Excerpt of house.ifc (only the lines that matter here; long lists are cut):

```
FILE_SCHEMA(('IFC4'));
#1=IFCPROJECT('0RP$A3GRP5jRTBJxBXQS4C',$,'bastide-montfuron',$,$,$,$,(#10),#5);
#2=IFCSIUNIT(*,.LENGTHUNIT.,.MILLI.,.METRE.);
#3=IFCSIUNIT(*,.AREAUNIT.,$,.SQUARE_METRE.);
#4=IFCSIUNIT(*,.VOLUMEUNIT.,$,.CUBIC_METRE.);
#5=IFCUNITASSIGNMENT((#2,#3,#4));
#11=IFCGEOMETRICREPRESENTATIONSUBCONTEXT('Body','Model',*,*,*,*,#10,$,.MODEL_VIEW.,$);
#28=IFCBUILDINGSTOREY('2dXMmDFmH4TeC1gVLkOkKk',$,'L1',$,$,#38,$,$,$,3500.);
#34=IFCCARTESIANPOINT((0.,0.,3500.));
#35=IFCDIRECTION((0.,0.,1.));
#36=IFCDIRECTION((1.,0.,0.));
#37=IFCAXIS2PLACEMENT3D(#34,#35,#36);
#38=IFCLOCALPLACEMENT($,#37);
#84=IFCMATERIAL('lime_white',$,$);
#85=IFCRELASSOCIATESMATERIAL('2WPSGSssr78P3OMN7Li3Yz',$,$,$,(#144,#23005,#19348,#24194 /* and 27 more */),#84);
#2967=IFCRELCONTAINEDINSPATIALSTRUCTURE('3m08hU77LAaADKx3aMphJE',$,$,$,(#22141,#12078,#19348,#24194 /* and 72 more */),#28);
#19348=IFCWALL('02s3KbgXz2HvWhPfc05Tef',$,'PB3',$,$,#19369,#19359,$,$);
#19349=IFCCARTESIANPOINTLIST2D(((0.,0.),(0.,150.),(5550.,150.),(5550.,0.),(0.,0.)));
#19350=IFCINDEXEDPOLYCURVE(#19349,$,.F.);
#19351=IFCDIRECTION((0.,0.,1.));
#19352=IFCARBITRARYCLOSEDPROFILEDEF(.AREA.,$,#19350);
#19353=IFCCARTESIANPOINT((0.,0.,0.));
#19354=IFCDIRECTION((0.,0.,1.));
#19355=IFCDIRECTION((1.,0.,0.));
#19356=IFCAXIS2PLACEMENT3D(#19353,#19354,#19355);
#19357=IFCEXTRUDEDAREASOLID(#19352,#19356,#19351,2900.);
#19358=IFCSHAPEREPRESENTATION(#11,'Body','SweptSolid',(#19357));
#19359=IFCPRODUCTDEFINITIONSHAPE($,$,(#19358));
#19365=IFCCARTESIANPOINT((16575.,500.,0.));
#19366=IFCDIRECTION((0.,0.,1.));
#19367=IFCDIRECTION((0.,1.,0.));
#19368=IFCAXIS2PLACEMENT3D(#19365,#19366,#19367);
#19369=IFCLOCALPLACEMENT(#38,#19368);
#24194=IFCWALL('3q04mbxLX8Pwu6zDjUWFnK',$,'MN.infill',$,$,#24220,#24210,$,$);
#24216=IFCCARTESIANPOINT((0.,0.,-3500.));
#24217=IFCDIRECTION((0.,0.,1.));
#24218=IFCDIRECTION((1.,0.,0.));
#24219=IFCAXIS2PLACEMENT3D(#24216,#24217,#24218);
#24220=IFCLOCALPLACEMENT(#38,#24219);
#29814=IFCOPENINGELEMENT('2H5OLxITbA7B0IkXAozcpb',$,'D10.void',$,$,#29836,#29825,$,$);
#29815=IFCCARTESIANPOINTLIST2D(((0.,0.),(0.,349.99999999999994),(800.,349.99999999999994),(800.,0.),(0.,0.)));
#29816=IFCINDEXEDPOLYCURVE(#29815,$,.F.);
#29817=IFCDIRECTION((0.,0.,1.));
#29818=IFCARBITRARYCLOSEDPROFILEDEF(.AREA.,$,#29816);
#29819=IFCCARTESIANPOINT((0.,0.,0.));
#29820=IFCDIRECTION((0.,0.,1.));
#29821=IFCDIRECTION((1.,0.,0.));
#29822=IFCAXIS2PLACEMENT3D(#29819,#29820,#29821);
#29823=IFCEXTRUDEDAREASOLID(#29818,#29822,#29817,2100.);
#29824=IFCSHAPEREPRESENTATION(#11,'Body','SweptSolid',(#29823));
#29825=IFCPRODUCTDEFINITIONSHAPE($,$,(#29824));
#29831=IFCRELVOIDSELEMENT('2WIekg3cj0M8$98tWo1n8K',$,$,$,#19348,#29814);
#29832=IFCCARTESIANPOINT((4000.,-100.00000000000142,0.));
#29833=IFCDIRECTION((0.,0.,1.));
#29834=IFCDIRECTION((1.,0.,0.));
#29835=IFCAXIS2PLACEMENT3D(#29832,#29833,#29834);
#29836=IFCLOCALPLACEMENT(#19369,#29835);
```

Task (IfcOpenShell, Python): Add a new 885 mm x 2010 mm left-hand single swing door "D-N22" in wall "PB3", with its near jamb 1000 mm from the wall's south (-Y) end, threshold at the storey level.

```python
import numpy as np
import ifcopenshell
import ifcopenshell.api.feature
import ifcopenshell.api.geometry
import ifcopenshell.api.root
import ifcopenshell.api.spatial
import ifcopenshell.geom
import ifcopenshell.util.element
import ifcopenshell.util.placement
import ifcopenshell.util.representation
import ifcopenshell.util.shape
import ifcopenshell.util.unit

model = ifcopenshell.open("house.ifc")
unit_scale = ifcopenshell.util.unit.calculate_unit_scale(model)
settings = ifcopenshell.geom.settings()


def volume(element):
    """Net volume in cubic metres, openings subtracted."""
    shape = ifcopenshell.geom.create_shape(settings, element)
    return ifcopenshell.util.shape.get_volume(shape.geometry)


wall = model.by_guid("02s3KbgXz2HvWhPfc05Tef")
storey = ifcopenshell.util.element.get_container(wall, ifc_class="IfcBuildingStorey")
context = ifcopenshell.util.representation.get_context(model, "Model", "Body", "MODEL_VIEW")
before = volume(wall)

width, height, from_end, sill = 0.885, 2.01, 1, 0.0  # metres

# The wall runs along its own X axis, and the end named is its -X end.
wall_shape = ifcopenshell.geom.create_shape(settings, wall)
x, y, z = ifcopenshell.util.shape.get_vertices(wall_shape.geometry).T
start = x.min() + from_end
face, thickness = float(y.min()), float(y.max() - y.min())
wall_matrix = ifcopenshell.util.placement.get_local_placement(wall.ObjectPlacement)
level = ifcopenshell.util.placement.get_local_placement(storey.ObjectPlacement)[2, 3]


def in_wall(x, y):
    """Placement at x, y metres in the wall's axes, at sill height."""
    matrix = wall_matrix.copy()
    matrix[:, 3] = wall_matrix @ np.array([x / unit_scale, y / unit_scale, 0.0, 1.0])
    matrix[2, 3] = level + sill / unit_scale
    return matrix


# Opening: a box that overshoots both wall faces by 50 mm.
opening = ifcopenshell.api.root.create_entity(model, ifc_class="IfcOpeningElement", predefined_type="OPENING")
box = ifcopenshell.api.geometry.add_wall_representation(
    model, context=context, length=width, height=height, thickness=thickness + 0.1
)
ifcopenshell.api.geometry.assign_representation(model, product=opening, representation=box)
ifcopenshell.api.geometry.edit_object_placement(model, product=opening, matrix=in_wall(start, face - 0.05), is_si=False)
ifcopenshell.api.feature.add_feature(model, feature=opening, element=wall)

door = ifcopenshell.api.root.create_entity(model, ifc_class="IfcDoor", name="D-N22", predefined_type="DOOR")
door.OverallWidth, door.OverallHeight = width / unit_scale, height / unit_scale
door.OperationType = "SINGLE_SWING_LEFT"
body = ifcopenshell.api.geometry.add_door_representation(
    model,
    context=context,
    overall_width=door.OverallWidth,
    overall_height=door.OverallHeight,
    operation_type="SINGLE_SWING_LEFT",
    lining_properties={"LiningDepth": thickness / unit_scale, "ThresholdDepth": thickness / unit_scale},
)
ifcopenshell.api.geometry.assign_representation(model, product=door, representation=body)
ifcopenshell.api.spatial.assign_container(model, products=[door], relating_structure=storey)
ifcopenshell.api.feature.add_filling(model, opening=opening, element=door)

# The lining spans the wall, so the door starts at the wall face.
ifcopenshell.api.geometry.edit_object_placement(model, product=door, matrix=in_wall(start, face), is_si=False)

after = volume(wall)

print(f"wall volume {before:.3f} -> {after:.3f} m3")

model.write("house_edited.ifc")
```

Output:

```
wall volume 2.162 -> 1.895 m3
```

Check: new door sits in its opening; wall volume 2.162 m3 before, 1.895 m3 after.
